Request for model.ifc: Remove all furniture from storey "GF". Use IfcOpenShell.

First a look at what the model holds.

```python
import ifcopenshell
import ifcopenshell.util.element

model = ifcopenshell.open("model.ifc")
print(model.schema)
storey = next(s for s in model.by_type("IfcBuildingStorey") if s.Name == "GF")
furniture = [e for e in ifcopenshell.util.element.get_decomposition(storey) if e.is_a("IfcFurnishingElement")]
seen = {}
for e in furniture:
    element_type = ifcopenshell.util.element.get_type(e)
    name = element_type.Name if element_type not in (None, e) else None
    seen[name] = seen.get(name, 0) + 1
for name, count in sorted(seen.items(), key=str):
    print(count, "x", name)
```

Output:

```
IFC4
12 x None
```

```python
import ifcopenshell
import ifcopenshell.api.root
import ifcopenshell.util.element

model = ifcopenshell.open("model.ifc")

storey = next(s for s in model.by_type("IfcBuildingStorey") if s.Name == "GF")
furniture = [e for e in ifcopenshell.util.element.get_decomposition(storey) if e.is_a("IfcFurnishingElement")]

for e in furniture:
    ifcopenshell.api.root.remove_product(model, product=e)
print(len(furniture), "removed")

model.write("model_edited.ifc")
```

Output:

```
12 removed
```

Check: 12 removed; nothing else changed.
